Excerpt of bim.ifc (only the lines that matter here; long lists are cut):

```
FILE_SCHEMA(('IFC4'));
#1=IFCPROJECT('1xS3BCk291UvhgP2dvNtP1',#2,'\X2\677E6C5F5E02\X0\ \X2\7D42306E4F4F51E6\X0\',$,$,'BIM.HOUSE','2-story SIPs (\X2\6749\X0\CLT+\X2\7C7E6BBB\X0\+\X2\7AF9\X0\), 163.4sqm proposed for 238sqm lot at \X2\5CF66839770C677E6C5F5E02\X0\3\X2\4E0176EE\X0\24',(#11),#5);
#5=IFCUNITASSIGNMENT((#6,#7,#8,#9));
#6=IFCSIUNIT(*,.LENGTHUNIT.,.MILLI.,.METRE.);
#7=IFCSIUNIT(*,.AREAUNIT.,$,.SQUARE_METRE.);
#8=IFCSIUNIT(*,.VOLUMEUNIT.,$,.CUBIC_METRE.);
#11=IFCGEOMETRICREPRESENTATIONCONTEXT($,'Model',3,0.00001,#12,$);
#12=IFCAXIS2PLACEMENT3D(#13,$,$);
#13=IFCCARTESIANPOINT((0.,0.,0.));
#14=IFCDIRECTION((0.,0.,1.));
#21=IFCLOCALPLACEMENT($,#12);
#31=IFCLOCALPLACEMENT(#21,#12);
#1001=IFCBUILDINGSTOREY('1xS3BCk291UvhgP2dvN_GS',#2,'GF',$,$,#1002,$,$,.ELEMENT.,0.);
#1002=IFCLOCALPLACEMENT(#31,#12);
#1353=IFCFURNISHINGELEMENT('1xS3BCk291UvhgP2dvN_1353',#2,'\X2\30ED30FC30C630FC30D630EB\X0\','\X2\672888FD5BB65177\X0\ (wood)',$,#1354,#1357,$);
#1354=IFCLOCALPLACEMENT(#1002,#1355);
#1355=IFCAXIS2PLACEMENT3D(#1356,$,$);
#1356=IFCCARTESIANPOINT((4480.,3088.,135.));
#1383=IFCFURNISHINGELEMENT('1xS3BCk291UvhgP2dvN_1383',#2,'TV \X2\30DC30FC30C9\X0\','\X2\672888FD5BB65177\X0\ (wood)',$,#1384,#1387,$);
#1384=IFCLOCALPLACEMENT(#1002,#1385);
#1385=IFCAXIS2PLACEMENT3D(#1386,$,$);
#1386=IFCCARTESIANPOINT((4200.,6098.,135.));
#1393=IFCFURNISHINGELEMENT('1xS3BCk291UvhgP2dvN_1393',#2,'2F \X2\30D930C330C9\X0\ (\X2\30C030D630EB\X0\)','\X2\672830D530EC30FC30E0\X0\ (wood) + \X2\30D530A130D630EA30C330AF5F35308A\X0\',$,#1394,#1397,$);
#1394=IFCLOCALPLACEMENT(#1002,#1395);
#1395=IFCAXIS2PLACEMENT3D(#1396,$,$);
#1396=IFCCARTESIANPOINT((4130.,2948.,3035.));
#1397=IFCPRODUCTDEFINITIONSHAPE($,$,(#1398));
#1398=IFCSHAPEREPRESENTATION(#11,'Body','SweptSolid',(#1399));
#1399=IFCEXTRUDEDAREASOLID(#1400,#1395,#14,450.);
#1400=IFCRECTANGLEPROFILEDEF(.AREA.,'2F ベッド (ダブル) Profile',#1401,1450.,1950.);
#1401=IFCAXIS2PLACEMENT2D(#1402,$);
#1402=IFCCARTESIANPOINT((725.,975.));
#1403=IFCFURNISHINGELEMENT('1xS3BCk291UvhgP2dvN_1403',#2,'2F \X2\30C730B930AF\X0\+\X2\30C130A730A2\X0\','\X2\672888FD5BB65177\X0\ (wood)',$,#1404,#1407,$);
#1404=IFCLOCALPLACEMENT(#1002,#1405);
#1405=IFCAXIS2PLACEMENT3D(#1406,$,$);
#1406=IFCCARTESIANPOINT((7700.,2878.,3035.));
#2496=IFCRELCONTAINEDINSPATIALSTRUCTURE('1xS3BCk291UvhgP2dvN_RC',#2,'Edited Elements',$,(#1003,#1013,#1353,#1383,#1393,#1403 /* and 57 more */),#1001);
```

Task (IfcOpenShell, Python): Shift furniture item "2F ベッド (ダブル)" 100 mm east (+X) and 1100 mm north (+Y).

```python
import ifcopenshell
import ifcopenshell.api.geometry
import ifcopenshell.util.placement
import ifcopenshell.util.unit

model = ifcopenshell.open("bim.ifc")
unit_scale = ifcopenshell.util.unit.calculate_unit_scale(model)

item = model.by_guid("1xS3BCk291UvhgP2dvN_1393")
matrix = ifcopenshell.util.placement.get_local_placement(item.ObjectPlacement)
matrix[0, 3] += 0.1 / unit_scale
matrix[1, 3] += 1.1 / unit_scale
ifcopenshell.api.geometry.edit_object_placement(model, product=item, matrix=matrix, is_si=False)

print(ifcopenshell.util.placement.get_local_placement(item.ObjectPlacement).round(3) + 0.0)

model.write("bim_rev.ifc")
```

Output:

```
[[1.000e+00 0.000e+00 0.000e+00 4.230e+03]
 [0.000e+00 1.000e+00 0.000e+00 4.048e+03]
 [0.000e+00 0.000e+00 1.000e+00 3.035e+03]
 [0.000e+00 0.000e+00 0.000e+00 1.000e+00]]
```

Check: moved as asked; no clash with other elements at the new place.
